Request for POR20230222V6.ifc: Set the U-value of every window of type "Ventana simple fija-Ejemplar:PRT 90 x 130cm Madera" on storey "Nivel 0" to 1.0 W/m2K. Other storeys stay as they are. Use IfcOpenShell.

First a look at what the model holds.

```python
import ifcopenshell
import ifcopenshell.util.element

model = ifcopenshell.open("POR20230222V6.ifc")
print(model.schema)
storey = next(s for s in model.by_type("IfcBuildingStorey") if s.Name == "Nivel 0")
windows = [e for e in ifcopenshell.util.element.get_decomposition(storey) if e.is_a("IfcWindow")]
seen = {}
for e in windows:
    element_type = ifcopenshell.util.element.get_type(e)
    key = (element_type.Name if element_type != e and element_type else None, ifcopenshell.util.element.get_pset(e, "Pset_WindowCommon", "ThermalTransmittance"))
    seen[key] = seen.get(key, 0) + 1
for (name, value), count in sorted(seen.items(), key=str):
    print(count, "x", name, "|", value)
```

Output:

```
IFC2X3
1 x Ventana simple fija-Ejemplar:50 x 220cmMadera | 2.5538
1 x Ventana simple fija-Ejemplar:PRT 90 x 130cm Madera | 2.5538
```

```python
import ifcopenshell
import ifcopenshell.api.pset
import ifcopenshell.util.element

model = ifcopenshell.open("POR20230222V6.ifc")

storey = next(s for s in model.by_type("IfcBuildingStorey") if s.Name == "Nivel 0")
windows = [e for e in ifcopenshell.util.element.get_decomposition(storey) if e.is_a("IfcWindow")]

count = 0
for e in windows:
    element_type = ifcopenshell.util.element.get_type(e)
    if element_type in (None, e) or element_type.Name != "Ventana simple fija-Ejemplar:PRT 90 x 130cm Madera":
        continue
    # add_pset returns the element's existing set when there is one.
    pset = ifcopenshell.api.pset.add_pset(model, product=e, name="Pset_WindowCommon")
    ifcopenshell.api.pset.edit_pset(model, pset=pset, properties={"ThermalTransmittance": 1.0})
    count += 1

print(count, "windows updated")

model.write("POR20230222V6_edited.ifc")
```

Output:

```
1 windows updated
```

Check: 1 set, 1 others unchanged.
